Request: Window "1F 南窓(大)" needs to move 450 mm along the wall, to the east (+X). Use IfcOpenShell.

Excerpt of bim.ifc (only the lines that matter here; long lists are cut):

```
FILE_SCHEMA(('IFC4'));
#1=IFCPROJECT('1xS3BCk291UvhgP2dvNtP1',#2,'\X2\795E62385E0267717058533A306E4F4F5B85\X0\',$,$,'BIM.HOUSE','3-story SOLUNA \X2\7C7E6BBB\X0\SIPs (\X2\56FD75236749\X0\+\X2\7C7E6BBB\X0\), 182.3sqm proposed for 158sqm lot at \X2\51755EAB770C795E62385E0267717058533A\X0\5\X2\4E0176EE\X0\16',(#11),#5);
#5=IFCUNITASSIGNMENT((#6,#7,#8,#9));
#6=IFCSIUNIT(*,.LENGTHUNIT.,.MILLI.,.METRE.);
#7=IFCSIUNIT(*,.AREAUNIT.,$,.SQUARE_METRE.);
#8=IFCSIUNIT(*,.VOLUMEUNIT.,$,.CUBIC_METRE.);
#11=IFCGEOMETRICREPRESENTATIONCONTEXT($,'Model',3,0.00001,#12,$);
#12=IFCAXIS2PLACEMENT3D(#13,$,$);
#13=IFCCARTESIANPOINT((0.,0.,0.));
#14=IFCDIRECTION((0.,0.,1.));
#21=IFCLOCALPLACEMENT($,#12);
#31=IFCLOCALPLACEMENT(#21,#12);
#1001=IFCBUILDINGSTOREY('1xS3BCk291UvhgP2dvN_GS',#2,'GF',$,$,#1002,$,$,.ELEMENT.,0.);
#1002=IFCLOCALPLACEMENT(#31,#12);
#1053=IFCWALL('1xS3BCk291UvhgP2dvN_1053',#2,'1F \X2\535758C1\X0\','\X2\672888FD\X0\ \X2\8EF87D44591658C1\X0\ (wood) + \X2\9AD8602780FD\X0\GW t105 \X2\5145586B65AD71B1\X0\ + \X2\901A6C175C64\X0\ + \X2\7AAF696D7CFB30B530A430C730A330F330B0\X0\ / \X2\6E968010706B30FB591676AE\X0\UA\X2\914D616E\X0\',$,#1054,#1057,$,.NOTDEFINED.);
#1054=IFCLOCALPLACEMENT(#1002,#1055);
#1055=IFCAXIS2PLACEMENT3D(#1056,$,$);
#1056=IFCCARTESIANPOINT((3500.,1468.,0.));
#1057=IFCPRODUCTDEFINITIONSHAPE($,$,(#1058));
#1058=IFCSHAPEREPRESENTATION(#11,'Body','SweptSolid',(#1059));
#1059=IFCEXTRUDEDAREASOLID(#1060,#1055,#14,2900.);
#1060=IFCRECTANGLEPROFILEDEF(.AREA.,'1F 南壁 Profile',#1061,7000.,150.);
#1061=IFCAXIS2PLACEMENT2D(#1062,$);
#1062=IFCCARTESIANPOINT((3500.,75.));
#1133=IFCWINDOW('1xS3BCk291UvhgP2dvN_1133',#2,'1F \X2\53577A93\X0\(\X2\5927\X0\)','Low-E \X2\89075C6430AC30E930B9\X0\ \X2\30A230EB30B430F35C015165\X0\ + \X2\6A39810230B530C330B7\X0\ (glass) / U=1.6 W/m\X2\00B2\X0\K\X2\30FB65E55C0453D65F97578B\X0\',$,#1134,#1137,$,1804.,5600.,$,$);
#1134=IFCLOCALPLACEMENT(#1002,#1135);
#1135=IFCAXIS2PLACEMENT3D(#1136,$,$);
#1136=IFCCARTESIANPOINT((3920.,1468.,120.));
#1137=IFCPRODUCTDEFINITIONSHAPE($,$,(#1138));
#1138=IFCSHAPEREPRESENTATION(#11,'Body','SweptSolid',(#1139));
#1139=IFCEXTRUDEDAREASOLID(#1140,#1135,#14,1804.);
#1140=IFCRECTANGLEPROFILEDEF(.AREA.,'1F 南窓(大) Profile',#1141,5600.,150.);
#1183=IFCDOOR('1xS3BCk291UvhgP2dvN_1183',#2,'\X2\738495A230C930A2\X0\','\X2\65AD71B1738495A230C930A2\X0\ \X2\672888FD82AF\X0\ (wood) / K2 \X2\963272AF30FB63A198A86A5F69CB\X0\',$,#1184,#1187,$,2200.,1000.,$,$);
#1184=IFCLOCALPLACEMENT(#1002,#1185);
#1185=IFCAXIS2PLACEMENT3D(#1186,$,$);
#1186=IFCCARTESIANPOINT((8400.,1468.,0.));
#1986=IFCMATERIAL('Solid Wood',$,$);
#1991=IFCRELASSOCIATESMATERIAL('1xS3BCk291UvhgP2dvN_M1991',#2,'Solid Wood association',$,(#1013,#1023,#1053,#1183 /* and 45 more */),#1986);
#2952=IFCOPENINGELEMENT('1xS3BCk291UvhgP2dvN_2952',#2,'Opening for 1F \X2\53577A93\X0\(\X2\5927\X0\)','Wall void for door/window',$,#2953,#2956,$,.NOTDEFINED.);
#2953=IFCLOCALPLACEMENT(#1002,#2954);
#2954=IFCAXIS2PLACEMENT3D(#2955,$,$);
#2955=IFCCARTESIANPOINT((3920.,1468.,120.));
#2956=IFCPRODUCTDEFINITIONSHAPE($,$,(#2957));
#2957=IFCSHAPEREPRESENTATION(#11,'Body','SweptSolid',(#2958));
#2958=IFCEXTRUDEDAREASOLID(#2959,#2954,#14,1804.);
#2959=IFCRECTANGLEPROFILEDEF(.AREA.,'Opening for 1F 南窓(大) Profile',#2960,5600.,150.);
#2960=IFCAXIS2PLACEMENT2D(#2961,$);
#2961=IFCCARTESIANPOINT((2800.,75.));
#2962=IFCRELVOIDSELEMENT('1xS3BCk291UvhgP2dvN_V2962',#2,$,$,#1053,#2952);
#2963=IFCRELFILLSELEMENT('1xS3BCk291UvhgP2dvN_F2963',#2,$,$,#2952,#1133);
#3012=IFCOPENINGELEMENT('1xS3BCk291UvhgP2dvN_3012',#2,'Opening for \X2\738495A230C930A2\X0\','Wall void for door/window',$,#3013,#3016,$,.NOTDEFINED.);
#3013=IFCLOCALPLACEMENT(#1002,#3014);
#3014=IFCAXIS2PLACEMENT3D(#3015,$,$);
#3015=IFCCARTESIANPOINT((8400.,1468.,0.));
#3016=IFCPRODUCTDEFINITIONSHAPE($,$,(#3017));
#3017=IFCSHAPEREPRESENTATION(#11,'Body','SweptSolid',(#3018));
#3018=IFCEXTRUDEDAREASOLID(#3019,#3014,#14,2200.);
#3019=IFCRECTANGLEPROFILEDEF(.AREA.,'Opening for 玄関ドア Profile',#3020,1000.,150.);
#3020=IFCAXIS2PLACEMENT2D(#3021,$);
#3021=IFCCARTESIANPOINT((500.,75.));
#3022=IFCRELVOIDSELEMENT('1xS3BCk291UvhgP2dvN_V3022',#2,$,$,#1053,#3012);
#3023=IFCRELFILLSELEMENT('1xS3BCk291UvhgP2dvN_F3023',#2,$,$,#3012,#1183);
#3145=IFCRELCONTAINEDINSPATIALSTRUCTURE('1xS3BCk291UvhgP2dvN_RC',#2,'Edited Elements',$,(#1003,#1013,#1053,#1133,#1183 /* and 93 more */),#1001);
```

```python
import ifcopenshell
import ifcopenshell.api.geometry
import ifcopenshell.util.placement
import ifcopenshell.util.unit

model = ifcopenshell.open("bim.ifc")
unit_scale = ifcopenshell.util.unit.calculate_unit_scale(model)

window = model.by_guid("1xS3BCk291UvhgP2dvN_1133")
opening = window.FillsVoids[0].RelatingOpeningElement
wall = opening.VoidsElements[0].RelatingBuildingElement

wall_matrix = ifcopenshell.util.placement.get_local_placement(wall.ObjectPlacement)
shift = wall_matrix[:3, 0] * 0.45 / unit_scale
before = ifcopenshell.util.placement.get_local_placement(window.ObjectPlacement)[:3, 3].copy()

# The window is not placed relative to its opening, so move both.
for product in (opening, window):
    matrix = ifcopenshell.util.placement.get_local_placement(product.ObjectPlacement)
    matrix[:3, 3] += shift
    ifcopenshell.api.geometry.edit_object_placement(model, product=product, matrix=matrix, is_si=False)

after = ifcopenshell.util.placement.get_local_placement(window.ObjectPlacement)[:3, 3]
print("window moved by", (after - before).round(3) + 0.0)

model.write("bim_edited.ifc")
```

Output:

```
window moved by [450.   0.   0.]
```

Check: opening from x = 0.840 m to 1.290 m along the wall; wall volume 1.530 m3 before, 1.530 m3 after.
